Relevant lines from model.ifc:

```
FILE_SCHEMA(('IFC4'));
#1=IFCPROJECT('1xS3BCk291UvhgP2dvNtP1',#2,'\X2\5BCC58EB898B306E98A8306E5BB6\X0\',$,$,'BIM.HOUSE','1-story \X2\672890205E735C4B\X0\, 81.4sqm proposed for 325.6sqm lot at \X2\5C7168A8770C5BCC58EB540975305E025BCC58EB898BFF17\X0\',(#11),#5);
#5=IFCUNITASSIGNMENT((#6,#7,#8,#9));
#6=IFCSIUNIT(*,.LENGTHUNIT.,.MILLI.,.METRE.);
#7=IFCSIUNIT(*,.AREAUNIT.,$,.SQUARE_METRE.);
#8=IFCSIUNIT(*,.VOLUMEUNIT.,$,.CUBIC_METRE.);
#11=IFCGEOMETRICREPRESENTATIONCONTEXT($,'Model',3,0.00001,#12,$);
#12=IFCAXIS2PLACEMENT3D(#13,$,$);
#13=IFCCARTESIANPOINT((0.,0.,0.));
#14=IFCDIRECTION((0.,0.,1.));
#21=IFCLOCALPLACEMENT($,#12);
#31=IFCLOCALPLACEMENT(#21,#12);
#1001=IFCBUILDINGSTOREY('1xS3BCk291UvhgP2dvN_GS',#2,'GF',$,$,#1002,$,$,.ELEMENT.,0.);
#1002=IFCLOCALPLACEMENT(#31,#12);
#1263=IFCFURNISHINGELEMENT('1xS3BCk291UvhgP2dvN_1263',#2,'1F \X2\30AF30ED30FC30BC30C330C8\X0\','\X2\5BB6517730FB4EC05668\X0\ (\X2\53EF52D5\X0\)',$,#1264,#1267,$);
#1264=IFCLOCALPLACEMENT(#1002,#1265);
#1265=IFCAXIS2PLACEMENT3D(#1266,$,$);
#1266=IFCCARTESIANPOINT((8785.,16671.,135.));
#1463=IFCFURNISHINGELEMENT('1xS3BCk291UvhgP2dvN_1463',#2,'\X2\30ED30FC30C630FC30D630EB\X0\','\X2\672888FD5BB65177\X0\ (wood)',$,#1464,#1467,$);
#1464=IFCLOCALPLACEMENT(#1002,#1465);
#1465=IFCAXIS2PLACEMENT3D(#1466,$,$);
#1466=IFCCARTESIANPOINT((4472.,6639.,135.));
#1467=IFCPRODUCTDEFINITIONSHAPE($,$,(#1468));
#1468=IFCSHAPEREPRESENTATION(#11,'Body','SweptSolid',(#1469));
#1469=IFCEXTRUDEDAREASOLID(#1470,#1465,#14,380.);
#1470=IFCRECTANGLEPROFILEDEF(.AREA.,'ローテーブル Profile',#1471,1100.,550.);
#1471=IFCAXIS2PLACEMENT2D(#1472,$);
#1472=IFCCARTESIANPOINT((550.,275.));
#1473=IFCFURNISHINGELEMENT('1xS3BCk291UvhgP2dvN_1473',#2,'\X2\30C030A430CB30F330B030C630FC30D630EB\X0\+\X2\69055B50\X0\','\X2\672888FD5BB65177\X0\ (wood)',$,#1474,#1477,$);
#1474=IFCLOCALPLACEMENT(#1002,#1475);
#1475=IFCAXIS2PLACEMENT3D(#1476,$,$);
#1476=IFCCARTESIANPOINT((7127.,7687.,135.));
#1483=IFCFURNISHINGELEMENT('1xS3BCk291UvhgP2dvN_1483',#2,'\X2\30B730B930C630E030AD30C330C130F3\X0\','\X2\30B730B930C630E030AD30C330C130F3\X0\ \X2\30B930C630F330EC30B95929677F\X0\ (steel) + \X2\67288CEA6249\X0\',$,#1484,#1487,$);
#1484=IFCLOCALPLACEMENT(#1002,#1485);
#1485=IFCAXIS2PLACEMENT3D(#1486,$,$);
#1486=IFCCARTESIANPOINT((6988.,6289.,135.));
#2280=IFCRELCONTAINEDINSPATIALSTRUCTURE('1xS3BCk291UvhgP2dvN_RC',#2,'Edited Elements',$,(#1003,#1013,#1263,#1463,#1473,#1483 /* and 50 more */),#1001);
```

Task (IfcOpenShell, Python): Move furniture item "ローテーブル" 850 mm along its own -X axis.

```python
import ifcopenshell
import ifcopenshell.api.geometry
import ifcopenshell.util.placement

model = ifcopenshell.open("model.ifc")

item = model.by_guid("1xS3BCk291UvhgP2dvN_1463")
matrix = ifcopenshell.util.placement.get_local_placement(item.ObjectPlacement)
matrix[:3, 3] -= matrix[:3, 0] * 850.0
ifcopenshell.api.geometry.edit_object_placement(model, product=item, matrix=matrix, is_si=False)

print(ifcopenshell.util.placement.get_local_placement(item.ObjectPlacement).round(3) + 0.0)

model.write("model-out.ifc")
```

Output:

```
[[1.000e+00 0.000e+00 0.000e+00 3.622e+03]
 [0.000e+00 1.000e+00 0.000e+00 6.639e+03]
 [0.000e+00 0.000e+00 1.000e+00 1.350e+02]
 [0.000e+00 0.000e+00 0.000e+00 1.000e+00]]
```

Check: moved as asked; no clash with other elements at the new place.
